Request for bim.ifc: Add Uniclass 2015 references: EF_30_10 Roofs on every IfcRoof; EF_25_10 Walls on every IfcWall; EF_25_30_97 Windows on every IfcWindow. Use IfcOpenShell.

First a look at what the model holds.

```python
import ifcopenshell

model = ifcopenshell.open("bim.ifc")
print(model.schema)
print("classifications:", [c.Name for c in model.by_type("IfcClassification")])
for ifc_class in ("IfcDoor", "IfcRoof", "IfcStair", "IfcWall", "IfcWindow"):
    print(ifc_class, len(model.by_type(ifc_class)))
```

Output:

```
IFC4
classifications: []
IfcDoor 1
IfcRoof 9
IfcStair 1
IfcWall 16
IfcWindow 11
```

```python
import ifcopenshell
import ifcopenshell.api.classification

model = ifcopenshell.open("bim.ifc")

system = ifcopenshell.api.classification.add_classification(model, classification="Uniclass 2015")

codes = {
    "IfcRoof": ("EF_30_10", "Roofs"),
    "IfcWall": ("EF_25_10", "Walls"),
    "IfcWindow": ("EF_25_30_97", "Windows"),
}
for ifc_class, (code, name) in codes.items():
    products = model.by_type(ifc_class)
    ifcopenshell.api.classification.add_reference(
        model, products=products, classification=system, identification=code, name=name
    )
    print(code, len(products))

model.write("bim-out.ifc")
```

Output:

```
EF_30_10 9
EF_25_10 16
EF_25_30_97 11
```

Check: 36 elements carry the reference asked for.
